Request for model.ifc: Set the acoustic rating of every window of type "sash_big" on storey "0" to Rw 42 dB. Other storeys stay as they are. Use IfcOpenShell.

First a look at what the model holds.

```python
import ifcopenshell
import ifcopenshell.util.element

model = ifcopenshell.open("model.ifc")
print(model.schema)
storey = next(s for s in model.by_type("IfcBuildingStorey") if s.Name == "0")
windows = [e for e in ifcopenshell.util.element.get_decomposition(storey) if e.is_a("IfcWindow")]
seen = {}
for e in windows:
    element_type = ifcopenshell.util.element.get_type(e)
    key = (element_type.Name if element_type != e and element_type else None, ifcopenshell.util.element.get_pset(e, "Pset_WindowCommon", "AcousticRating"))
    seen[key] = seen.get(key, 0) + 1
for (name, value), count in sorted(seen.items(), key=str):
    print(count, "x", name, "|", value)
```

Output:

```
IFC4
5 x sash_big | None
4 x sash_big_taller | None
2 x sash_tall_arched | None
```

```python
import ifcopenshell
import ifcopenshell.api.pset
import ifcopenshell.util.element

model = ifcopenshell.open("model.ifc")

storey = next(s for s in model.by_type("IfcBuildingStorey") if s.Name == "0")
windows = [e for e in ifcopenshell.util.element.get_decomposition(storey) if e.is_a("IfcWindow")]

count = 0
for e in windows:
    element_type = ifcopenshell.util.element.get_type(e)
    if element_type in (None, e) or element_type.Name != "sash_big":
        continue
    # add_pset returns the element's existing set when there is one.
    pset = ifcopenshell.api.pset.add_pset(model, product=e, name="Pset_WindowCommon")
    ifcopenshell.api.pset.edit_pset(model, pset=pset, properties={"AcousticRating": "Rw 42 dB"})
    count += 1

print(count, "windows updated")

model.write("model-out.ifc")
```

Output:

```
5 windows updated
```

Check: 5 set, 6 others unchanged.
